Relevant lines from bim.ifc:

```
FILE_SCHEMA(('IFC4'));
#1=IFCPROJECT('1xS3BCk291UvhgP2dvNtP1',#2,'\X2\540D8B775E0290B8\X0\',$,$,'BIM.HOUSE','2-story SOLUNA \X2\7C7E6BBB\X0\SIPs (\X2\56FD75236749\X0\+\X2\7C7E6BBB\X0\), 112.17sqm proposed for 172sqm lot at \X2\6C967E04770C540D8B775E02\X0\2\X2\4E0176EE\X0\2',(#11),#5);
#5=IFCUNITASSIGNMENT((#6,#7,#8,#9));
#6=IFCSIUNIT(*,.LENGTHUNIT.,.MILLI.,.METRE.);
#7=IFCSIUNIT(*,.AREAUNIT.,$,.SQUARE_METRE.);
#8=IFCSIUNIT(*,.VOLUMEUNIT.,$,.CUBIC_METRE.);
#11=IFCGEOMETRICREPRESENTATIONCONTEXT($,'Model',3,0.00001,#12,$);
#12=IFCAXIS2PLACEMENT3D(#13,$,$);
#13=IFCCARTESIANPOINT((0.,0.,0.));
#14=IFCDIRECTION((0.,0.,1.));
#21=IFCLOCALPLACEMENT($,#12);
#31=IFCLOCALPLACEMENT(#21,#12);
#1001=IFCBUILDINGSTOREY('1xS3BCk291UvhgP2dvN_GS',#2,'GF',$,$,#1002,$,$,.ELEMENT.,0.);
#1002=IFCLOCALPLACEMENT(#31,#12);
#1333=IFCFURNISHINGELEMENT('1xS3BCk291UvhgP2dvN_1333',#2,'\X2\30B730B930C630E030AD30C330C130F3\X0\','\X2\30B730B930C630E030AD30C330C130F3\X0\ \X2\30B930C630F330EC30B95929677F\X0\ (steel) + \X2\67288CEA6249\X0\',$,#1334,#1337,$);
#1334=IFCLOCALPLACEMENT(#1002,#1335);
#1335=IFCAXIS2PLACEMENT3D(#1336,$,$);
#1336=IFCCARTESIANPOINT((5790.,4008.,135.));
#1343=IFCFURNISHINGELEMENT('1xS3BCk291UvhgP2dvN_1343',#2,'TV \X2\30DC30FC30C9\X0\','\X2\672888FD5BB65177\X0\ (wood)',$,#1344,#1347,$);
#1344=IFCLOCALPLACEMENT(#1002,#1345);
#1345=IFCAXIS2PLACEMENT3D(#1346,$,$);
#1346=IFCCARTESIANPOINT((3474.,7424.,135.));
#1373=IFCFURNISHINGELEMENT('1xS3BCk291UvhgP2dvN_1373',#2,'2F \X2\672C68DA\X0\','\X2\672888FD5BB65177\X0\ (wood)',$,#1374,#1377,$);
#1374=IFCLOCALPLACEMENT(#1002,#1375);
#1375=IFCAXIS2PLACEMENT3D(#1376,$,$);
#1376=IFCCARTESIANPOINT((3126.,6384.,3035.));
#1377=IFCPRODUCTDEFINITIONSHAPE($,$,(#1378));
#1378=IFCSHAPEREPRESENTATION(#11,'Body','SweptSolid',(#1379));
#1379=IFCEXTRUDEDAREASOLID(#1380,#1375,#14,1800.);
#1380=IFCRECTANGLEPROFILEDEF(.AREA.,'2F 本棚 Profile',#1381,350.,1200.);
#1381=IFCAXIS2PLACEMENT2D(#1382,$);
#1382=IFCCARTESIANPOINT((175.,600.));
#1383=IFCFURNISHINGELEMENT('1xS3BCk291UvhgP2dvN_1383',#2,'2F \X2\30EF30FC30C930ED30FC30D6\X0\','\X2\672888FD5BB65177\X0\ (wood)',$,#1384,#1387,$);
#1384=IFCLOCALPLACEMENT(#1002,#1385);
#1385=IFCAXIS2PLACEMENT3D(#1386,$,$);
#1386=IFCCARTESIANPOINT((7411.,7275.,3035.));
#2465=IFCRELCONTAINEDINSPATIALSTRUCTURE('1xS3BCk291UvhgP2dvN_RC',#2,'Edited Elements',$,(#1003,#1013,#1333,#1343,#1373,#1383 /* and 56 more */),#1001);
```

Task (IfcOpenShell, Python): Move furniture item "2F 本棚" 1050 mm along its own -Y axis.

```python
import ifcopenshell
import ifcopenshell.api.geometry
import ifcopenshell.util.placement
import ifcopenshell.util.unit

model = ifcopenshell.open("bim.ifc")
unit_scale = ifcopenshell.util.unit.calculate_unit_scale(model)

item = model.by_id(1373)
matrix = ifcopenshell.util.placement.get_local_placement(item.ObjectPlacement)
matrix[:3, 3] -= matrix[:3, 1] * 1.05 / unit_scale
ifcopenshell.api.geometry.edit_object_placement(model, product=item, matrix=matrix, is_si=False)

print(ifcopenshell.util.placement.get_local_placement(item.ObjectPlacement).round(3) + 0.0)

model.write("bim_updated.ifc")
```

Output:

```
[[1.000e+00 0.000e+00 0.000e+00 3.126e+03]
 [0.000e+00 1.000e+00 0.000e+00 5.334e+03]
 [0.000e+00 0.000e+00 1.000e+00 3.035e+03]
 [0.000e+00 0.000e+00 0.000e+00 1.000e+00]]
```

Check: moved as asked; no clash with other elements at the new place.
